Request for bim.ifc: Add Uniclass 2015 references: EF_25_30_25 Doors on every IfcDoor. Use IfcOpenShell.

First a look at what the model holds.

```python
import ifcopenshell

model = ifcopenshell.open("bim.ifc")
print(model.schema)
print("classifications:", [c.Name for c in model.by_type("IfcClassification")])
for ifc_class in ("IfcDoor", "IfcRoof", "IfcStair", "IfcWall", "IfcWindow"):
    print(ifc_class, len(model.by_type(ifc_class)))
```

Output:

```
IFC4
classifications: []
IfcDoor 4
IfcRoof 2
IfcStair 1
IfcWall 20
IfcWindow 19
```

```python
import ifcopenshell
import ifcopenshell.api.classification

model = ifcopenshell.open("bim.ifc")

system = ifcopenshell.api.classification.add_classification(model, classification="Uniclass 2015")

codes = {
    "IfcDoor": ("EF_25_30_25", "Doors"),
}
for ifc_class, (code, name) in codes.items():
    products = model.by_type(ifc_class)
    ifcopenshell.api.classification.add_reference(
        model, products=products, classification=system, identification=code, name=name
    )
    print(code, len(products))

model.write("bim_rev.ifc")
```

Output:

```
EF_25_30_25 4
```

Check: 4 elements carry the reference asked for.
